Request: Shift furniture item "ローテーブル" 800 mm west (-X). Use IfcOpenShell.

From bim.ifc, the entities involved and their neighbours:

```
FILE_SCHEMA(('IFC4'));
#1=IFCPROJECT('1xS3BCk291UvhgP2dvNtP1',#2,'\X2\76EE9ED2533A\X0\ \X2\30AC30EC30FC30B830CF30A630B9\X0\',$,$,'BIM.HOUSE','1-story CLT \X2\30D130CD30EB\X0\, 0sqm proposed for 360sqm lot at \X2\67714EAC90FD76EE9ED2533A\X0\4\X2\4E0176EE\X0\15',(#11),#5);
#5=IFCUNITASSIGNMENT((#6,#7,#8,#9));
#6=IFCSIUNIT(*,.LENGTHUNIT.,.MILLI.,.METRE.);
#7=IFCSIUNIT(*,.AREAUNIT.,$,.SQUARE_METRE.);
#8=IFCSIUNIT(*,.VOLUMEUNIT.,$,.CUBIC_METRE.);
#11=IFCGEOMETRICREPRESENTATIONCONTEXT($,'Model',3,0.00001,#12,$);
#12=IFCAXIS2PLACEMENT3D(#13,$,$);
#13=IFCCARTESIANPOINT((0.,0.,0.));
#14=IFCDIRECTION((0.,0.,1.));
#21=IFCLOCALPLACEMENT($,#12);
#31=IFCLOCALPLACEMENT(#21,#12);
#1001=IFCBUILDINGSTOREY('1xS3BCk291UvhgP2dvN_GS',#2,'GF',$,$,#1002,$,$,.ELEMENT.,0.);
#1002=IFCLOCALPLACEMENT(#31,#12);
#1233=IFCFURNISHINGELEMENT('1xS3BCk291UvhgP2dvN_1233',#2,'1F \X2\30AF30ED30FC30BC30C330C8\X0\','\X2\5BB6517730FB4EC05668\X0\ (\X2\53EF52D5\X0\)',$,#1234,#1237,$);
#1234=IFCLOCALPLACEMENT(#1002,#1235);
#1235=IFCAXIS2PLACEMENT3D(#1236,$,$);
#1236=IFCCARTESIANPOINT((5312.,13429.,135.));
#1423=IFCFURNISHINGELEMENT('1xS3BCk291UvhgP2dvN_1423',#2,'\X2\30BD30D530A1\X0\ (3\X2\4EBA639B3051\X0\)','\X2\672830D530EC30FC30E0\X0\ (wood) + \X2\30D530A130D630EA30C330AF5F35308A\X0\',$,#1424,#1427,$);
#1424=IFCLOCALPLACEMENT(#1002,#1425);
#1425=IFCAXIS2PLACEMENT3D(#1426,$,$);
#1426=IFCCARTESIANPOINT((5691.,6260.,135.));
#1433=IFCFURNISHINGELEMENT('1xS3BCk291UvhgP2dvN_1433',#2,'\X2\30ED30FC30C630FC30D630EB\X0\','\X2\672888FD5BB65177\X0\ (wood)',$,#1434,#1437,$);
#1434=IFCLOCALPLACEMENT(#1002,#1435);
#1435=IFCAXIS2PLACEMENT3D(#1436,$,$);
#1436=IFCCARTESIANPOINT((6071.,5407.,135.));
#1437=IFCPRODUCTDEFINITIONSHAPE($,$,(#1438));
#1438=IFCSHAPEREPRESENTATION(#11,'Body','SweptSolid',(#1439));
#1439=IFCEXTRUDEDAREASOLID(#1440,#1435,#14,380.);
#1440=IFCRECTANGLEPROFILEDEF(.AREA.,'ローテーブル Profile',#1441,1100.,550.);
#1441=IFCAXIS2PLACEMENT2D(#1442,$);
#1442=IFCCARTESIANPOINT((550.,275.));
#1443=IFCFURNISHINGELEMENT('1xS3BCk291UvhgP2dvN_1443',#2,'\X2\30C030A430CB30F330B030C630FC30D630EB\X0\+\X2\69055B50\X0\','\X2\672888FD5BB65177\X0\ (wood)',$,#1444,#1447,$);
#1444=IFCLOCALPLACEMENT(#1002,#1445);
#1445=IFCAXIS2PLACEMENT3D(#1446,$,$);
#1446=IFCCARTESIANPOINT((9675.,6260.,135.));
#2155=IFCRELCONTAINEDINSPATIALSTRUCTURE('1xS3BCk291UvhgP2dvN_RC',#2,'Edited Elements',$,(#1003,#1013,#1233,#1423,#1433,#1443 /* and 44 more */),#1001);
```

```python
import ifcopenshell
import ifcopenshell.api.geometry
import ifcopenshell.util.placement
import ifcopenshell.util.unit

model = ifcopenshell.open("bim.ifc")
unit_scale = ifcopenshell.util.unit.calculate_unit_scale(model)

item = model.by_guid("1xS3BCk291UvhgP2dvN_1433")
matrix = ifcopenshell.util.placement.get_local_placement(item.ObjectPlacement)
matrix[0, 3] -= 0.8 / unit_scale
ifcopenshell.api.geometry.edit_object_placement(model, product=item, matrix=matrix, is_si=False)

print(ifcopenshell.util.placement.get_local_placement(item.ObjectPlacement).round(3) + 0.0)

model.write("bim-out.ifc")
```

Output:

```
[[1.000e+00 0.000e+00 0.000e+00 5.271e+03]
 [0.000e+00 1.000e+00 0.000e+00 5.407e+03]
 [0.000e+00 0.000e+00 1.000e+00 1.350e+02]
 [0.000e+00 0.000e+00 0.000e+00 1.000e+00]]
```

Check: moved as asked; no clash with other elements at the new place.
